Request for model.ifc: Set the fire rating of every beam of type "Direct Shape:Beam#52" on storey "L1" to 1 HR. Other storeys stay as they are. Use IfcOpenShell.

First a look at what the model holds.

```python
import ifcopenshell
import ifcopenshell.util.element

model = ifcopenshell.open("model.ifc")
print(model.schema)
storey = next(s for s in model.by_type("IfcBuildingStorey") if s.Name == "L1")
beams = [e for e in ifcopenshell.util.element.get_decomposition(storey) if e.is_a("IfcBeam")]
seen = {}
for e in beams:
    element_type = ifcopenshell.util.element.get_type(e)
    key = (element_type.Name if element_type != e and element_type else None, ifcopenshell.util.element.get_pset(e, "Pset_BeamCommon", "FireRating"))
    seen[key] = seen.get(key, 0) + 1
for (name, value), count in sorted(seen.items(), key=str):
    print(count, "x", name, "|", value)
```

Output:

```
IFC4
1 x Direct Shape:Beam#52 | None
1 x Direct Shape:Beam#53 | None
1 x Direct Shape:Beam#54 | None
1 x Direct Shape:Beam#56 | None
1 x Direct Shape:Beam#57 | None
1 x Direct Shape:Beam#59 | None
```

```python
import ifcopenshell
import ifcopenshell.api.pset
import ifcopenshell.util.element

model = ifcopenshell.open("model.ifc")

storey = next(s for s in model.by_type("IfcBuildingStorey") if s.Name == "L1")
beams = [e for e in ifcopenshell.util.element.get_decomposition(storey) if e.is_a("IfcBeam")]

count = 0
for e in beams:
    element_type = ifcopenshell.util.element.get_type(e)
    if element_type in (None, e) or element_type.Name != "Direct Shape:Beam#52":
        continue
    # add_pset returns the element's existing set when there is one.
    pset = ifcopenshell.api.pset.add_pset(model, product=e, name="Pset_BeamCommon")
    ifcopenshell.api.pset.edit_pset(model, pset=pset, properties={"FireRating": "1 HR"})
    count += 1

print(count, "beams updated")

model.write("model_updated.ifc")
```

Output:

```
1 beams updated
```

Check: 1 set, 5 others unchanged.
